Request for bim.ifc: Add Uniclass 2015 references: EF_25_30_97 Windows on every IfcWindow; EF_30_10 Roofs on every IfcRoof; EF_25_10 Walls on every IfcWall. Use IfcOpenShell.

First a look at what the model holds.

```python
import ifcopenshell

model = ifcopenshell.open("bim.ifc")
print(model.schema)
print("classifications:", [c.Name for c in model.by_type("IfcClassification")])
for ifc_class in ("IfcDoor", "IfcRoof", "IfcStair", "IfcWall", "IfcWindow"):
    print(ifc_class, len(model.by_type(ifc_class)))
```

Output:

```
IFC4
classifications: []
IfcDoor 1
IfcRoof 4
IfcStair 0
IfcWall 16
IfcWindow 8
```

```python
import ifcopenshell
import ifcopenshell.api.classification

model = ifcopenshell.open("bim.ifc")

system = ifcopenshell.api.classification.add_classification(model, classification="Uniclass 2015")

codes = {
    "IfcWindow": ("EF_25_30_97", "Windows"),
    "IfcRoof": ("EF_30_10", "Roofs"),
    "IfcWall": ("EF_25_10", "Walls"),
}
for ifc_class, (code, name) in codes.items():
    products = model.by_type(ifc_class)
    ifcopenshell.api.classification.add_reference(
        model, products=products, classification=system, identification=code, name=name
    )
    print(code, len(products))

model.write("bim_rev.ifc")
```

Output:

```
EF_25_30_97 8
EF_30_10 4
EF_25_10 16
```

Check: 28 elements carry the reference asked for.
